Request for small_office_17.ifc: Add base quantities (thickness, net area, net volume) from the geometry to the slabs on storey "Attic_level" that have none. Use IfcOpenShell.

First a look at what the model holds.

```python
import ifcopenshell
import ifcopenshell.util.element
import ifcopenshell.util.unit

model = ifcopenshell.open("small_office_17.ifc")
print(model.schema)
for unit_type in ("LENGTHUNIT", "AREAUNIT", "VOLUMEUNIT"):
    print(unit_type, ifcopenshell.util.unit.calculate_unit_scale(model, unit_type))
storey = next(s for s in model.by_type("IfcBuildingStorey") if s.Name == "Attic_level")
slabs = [e for e in ifcopenshell.util.element.get_decomposition(storey) if e.is_a("IfcSlab")]
for e in sorted(slabs, key=lambda e: e.id()):
    print(e.id(), e.is_a(), e.Name, list(ifcopenshell.util.element.get_psets(e, qtos_only=True)), sep=" | ")
```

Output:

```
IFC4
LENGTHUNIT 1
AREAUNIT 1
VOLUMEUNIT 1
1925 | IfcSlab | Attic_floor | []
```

```python
import ifcopenshell
import ifcopenshell.api.pset
import ifcopenshell.geom
import ifcopenshell.util.element
import ifcopenshell.util.shape
import ifcopenshell.util.unit

model = ifcopenshell.open("small_office_17.ifc")
unit_scale = ifcopenshell.util.unit.calculate_unit_scale(model)
area_scale = ifcopenshell.util.unit.calculate_unit_scale(model, "AREAUNIT")
volume_scale = ifcopenshell.util.unit.calculate_unit_scale(model, "VOLUMEUNIT")
settings = ifcopenshell.geom.settings()

storey = next(s for s in model.by_type("IfcBuildingStorey") if s.Name == "Attic_level")
slabs = [e for e in ifcopenshell.util.element.get_decomposition(storey) if e.is_a("IfcSlab")]

for e in sorted(slabs, key=lambda e: e.id()):
    if ifcopenshell.util.element.get_psets(e, qtos_only=True, should_inherit=False):
        continue
    # Geometry comes back in metres, in the element's own axes.
    shape = ifcopenshell.geom.create_shape(settings, e)
    values = {
        "Width": ifcopenshell.util.shape.get_z(shape.geometry) / unit_scale,
        "NetArea": ifcopenshell.util.shape.get_footprint_area(shape.geometry) / area_scale,
        "NetVolume": ifcopenshell.util.shape.get_volume(shape.geometry) / volume_scale,
    }
    qto = ifcopenshell.api.pset.add_qto(model, product=e, name="Qto_SlabBaseQuantities")
    ifcopenshell.api.pset.edit_qto(model, qto=qto, properties=values)
    print(e.id(), {k: round(v, 3) for k, v in values.items()})

model.write("small_office_17_edited.ifc")
```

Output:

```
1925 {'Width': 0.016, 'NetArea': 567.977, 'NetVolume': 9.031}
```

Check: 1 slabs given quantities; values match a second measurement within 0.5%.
